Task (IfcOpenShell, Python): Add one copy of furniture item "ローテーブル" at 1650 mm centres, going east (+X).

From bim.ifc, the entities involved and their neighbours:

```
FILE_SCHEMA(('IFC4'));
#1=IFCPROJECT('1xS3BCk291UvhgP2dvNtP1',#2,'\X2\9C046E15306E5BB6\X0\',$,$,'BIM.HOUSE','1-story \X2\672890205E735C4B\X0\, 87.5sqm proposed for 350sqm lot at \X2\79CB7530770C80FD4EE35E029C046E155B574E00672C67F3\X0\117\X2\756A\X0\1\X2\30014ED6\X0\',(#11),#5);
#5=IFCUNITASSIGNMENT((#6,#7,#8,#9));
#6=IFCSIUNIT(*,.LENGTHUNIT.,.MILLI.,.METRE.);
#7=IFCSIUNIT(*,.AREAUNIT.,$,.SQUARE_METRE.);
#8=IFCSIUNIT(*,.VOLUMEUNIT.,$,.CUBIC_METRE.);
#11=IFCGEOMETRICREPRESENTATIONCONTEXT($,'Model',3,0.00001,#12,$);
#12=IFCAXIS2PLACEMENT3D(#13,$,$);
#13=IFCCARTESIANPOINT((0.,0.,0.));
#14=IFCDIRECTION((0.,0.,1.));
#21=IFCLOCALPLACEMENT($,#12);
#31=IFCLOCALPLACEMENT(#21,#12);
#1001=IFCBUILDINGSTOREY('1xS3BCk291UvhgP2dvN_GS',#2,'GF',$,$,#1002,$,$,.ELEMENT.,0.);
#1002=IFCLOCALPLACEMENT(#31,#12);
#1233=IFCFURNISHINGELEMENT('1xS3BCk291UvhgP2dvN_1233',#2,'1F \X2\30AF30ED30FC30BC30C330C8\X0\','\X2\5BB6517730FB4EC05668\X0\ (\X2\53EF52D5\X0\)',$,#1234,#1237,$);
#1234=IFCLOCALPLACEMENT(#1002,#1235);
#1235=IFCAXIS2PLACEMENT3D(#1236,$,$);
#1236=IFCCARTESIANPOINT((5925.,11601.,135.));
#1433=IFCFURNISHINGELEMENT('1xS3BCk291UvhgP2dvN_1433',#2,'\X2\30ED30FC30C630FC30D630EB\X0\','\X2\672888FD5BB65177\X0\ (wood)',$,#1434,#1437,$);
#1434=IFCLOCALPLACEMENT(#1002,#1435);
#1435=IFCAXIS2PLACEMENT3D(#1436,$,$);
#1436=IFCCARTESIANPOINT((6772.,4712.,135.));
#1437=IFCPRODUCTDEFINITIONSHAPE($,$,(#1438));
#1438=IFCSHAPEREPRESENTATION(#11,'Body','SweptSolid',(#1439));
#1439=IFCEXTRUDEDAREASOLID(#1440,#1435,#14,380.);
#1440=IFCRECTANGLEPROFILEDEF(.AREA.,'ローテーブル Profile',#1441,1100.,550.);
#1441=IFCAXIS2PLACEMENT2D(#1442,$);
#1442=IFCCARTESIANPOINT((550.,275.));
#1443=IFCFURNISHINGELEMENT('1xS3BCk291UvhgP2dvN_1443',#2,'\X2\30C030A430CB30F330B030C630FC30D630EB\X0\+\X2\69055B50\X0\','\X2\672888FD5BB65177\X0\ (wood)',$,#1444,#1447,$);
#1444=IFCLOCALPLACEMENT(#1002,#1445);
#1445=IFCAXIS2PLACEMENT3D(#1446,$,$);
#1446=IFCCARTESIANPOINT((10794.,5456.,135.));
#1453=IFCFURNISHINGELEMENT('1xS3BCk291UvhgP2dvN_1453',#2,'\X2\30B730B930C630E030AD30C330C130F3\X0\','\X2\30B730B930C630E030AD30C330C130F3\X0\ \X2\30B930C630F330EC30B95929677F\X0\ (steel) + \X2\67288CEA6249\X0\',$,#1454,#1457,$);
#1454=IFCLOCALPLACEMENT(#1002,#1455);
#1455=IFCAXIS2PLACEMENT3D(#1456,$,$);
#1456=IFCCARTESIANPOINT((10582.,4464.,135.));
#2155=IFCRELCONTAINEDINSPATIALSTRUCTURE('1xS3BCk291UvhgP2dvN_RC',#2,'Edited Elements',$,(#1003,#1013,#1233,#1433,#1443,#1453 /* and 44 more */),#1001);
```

```python
import numpy as np
import ifcopenshell
import ifcopenshell.api.geometry
import ifcopenshell.api.root
import ifcopenshell.util.element
import ifcopenshell.util.placement
import ifcopenshell.util.unit

model = ifcopenshell.open("bim.ifc")
unit_scale = ifcopenshell.util.unit.calculate_unit_scale(model)


def reuse_history(source, copy):
    """copy_class also copies each property set's owner history, people and application; keep the originals."""
    for rel in copy.IsDefinedBy:
        if rel.is_a("IfcRelDefinesByProperties") and (history := rel.RelatingPropertyDefinition.OwnerHistory):
            rel.RelatingPropertyDefinition.OwnerHistory = source.OwnerHistory
            ifcopenshell.util.element.remove_deep2(model, history)


source = model.by_guid("1xS3BCk291UvhgP2dvN_1433")
base = ifcopenshell.util.placement.get_local_placement(source.ObjectPlacement)
step = np.array([1.0, 0.0, 0.0]) * 1.65 / unit_scale

for i in range(1, 2):
    copy = ifcopenshell.api.root.copy_class(model, product=source)
    copy.Representation = ifcopenshell.util.element.copy_deep(
        model, source.Representation, exclude=["IfcGeometricRepresentationContext", "IfcRepresentationMap"]
    )
    reuse_history(source, copy)
    matrix = base.copy()
    matrix[:3, 3] += i * step
    print("added at", matrix[:3, 3].round(3) + 0.0)
    ifcopenshell.api.geometry.edit_object_placement(model, product=copy, matrix=matrix, is_si=False)

model.write("bim_updated.ifc")
```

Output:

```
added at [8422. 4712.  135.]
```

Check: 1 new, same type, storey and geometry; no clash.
